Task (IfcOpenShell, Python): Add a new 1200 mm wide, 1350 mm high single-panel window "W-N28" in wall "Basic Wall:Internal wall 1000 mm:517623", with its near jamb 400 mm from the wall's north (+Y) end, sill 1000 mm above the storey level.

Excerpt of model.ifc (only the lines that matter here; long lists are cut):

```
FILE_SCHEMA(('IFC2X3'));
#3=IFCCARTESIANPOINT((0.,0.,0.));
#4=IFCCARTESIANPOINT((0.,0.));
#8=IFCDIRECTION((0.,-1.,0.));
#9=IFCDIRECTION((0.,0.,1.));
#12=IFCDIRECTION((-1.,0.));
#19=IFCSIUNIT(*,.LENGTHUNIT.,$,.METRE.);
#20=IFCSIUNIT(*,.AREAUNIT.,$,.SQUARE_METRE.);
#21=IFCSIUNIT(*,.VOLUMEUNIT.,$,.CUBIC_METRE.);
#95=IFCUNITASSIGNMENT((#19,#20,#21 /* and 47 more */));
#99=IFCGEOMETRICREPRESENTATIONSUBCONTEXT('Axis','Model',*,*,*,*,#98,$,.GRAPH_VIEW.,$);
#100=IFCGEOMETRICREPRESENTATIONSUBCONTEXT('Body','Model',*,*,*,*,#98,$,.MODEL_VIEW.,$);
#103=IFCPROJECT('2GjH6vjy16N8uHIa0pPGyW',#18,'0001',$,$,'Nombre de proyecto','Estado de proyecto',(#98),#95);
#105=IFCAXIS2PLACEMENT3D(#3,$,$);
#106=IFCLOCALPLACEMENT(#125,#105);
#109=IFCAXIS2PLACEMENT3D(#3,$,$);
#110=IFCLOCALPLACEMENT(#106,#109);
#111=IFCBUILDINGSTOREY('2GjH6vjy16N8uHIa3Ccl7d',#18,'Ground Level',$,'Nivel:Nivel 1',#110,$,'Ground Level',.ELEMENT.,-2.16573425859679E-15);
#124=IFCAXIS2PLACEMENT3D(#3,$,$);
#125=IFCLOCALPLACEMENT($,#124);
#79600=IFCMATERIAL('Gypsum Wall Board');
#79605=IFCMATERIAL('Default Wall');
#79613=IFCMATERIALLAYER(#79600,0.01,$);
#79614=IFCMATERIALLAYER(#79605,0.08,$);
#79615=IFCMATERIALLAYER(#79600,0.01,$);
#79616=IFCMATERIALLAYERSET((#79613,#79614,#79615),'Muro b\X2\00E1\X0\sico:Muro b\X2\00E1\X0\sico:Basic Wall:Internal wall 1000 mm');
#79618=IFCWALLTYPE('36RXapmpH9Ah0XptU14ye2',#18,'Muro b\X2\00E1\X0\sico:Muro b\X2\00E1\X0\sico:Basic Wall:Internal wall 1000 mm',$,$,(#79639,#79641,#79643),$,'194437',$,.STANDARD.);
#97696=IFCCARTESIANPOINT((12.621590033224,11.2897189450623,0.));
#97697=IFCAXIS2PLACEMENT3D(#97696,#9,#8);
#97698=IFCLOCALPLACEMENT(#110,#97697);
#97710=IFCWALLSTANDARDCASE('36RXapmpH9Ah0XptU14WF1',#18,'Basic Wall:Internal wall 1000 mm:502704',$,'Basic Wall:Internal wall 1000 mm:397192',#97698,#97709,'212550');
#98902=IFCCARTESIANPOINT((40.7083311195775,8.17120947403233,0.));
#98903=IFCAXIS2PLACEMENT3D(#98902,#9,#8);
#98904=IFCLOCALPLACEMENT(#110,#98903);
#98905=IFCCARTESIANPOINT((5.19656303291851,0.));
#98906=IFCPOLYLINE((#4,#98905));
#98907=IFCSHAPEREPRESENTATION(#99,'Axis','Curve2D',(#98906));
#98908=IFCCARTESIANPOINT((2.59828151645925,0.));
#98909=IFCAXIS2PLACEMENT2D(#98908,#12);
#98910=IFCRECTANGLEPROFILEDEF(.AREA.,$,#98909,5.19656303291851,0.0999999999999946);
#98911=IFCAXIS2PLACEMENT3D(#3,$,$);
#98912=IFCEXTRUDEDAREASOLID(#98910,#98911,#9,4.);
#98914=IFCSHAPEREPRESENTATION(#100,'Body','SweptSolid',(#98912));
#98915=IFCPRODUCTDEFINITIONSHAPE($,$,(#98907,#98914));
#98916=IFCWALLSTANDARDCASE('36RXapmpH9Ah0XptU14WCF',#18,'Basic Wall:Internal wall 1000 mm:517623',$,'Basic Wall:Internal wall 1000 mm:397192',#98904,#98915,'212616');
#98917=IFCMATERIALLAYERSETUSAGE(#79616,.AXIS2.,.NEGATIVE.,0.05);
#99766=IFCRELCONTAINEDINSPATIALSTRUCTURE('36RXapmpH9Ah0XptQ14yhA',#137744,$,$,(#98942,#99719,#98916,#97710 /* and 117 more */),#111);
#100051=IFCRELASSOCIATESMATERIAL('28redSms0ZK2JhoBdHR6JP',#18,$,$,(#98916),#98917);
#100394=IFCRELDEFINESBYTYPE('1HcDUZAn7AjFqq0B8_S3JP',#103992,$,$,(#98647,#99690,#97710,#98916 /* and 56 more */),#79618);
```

```python
import numpy as np
import ifcopenshell
import ifcopenshell.api.feature
import ifcopenshell.api.geometry
import ifcopenshell.api.root
import ifcopenshell.api.spatial
import ifcopenshell.api.type
import ifcopenshell.geom
import ifcopenshell.util.element
import ifcopenshell.util.placement
import ifcopenshell.util.representation
import ifcopenshell.util.shape
import ifcopenshell.util.unit

model = ifcopenshell.open("model.ifc")
unit_scale = ifcopenshell.util.unit.calculate_unit_scale(model)
settings = ifcopenshell.geom.settings()


def volume(element):
    """Net volume in cubic metres, openings subtracted."""
    shape = ifcopenshell.geom.create_shape(settings, element)
    return ifcopenshell.util.shape.get_volume(shape.geometry)


wall = model.by_guid("36RXapmpH9Ah0XptU14WCF")
storey = ifcopenshell.util.element.get_container(wall, ifc_class="IfcBuildingStorey")
context = ifcopenshell.util.representation.get_context(model, "Model", "Body", "MODEL_VIEW")
before = volume(wall)

width, height, from_end, sill = 1.2, 1.35, 0.4, 1  # metres

# The wall runs along its own X axis, and the end named is its -X end.
wall_shape = ifcopenshell.geom.create_shape(settings, wall)
x, y, z = ifcopenshell.util.shape.get_vertices(wall_shape.geometry).T
start = x.min() + from_end
face, thickness = float(y.min()), float(y.max() - y.min())
wall_matrix = ifcopenshell.util.placement.get_local_placement(wall.ObjectPlacement)
level = ifcopenshell.util.placement.get_local_placement(storey.ObjectPlacement)[2, 3]


def in_wall(x, y):
    """Placement at x, y metres in the wall's axes, at sill height."""
    matrix = wall_matrix.copy()
    matrix[:, 3] = wall_matrix @ np.array([x / unit_scale, y / unit_scale, 0.0, 1.0])
    matrix[2, 3] = level + sill / unit_scale
    return matrix


# Opening: a box that overshoots both wall faces by 50 mm.
opening = ifcopenshell.api.root.create_entity(model, ifc_class="IfcOpeningElement")
box = ifcopenshell.api.geometry.add_wall_representation(
    model, context=context, length=width, height=height, thickness=thickness + 0.1
)
ifcopenshell.api.geometry.assign_representation(model, product=opening, representation=box)
ifcopenshell.api.geometry.edit_object_placement(model, product=opening, matrix=in_wall(start, face - 0.05), is_si=False)
ifcopenshell.api.feature.add_feature(model, feature=opening, element=wall)

window = ifcopenshell.api.root.create_entity(model, ifc_class="IfcWindow", name="W-N28")
window.OverallWidth, window.OverallHeight = width / unit_scale, height / unit_scale
body = ifcopenshell.api.geometry.add_window_representation(
    model,
    context=context,
    overall_width=window.OverallWidth,
    overall_height=window.OverallHeight,
    partition_type="SINGLE_PANEL",
)
ifcopenshell.api.geometry.assign_representation(model, product=window, representation=body)
ifcopenshell.api.spatial.assign_container(model, products=[window], relating_structure=storey)
fills = ifcopenshell.api.feature.add_filling(model, opening=opening, element=window)
fills.OwnerHistory = window.OwnerHistory  # required in IFC2X3

# IFC2X3 keeps the operation on the window style.
style = ifcopenshell.api.root.create_entity(model, ifc_class="IfcWindowStyle", name="W-N28")
style.OperationType, style.ConstructionType = "SINGLE_PANEL", "NOTDEFINED"
style.ParameterTakesPrecedence = style.Sizeable = False
ifcopenshell.api.type.assign_type(model, related_objects=[window], relating_type=style)

# Centre the window in the wall's thickness.
ifcopenshell.api.geometry.edit_object_placement(model, product=window, matrix=in_wall(start, face), is_si=False)
window_shape = ifcopenshell.geom.create_shape(settings, window)
depth = ifcopenshell.util.shape.get_vertices(window_shape.geometry)[:, 1]
offset = face + thickness / 2 - (depth.min() + depth.max()) / 2
ifcopenshell.api.geometry.edit_object_placement(model, product=window, matrix=in_wall(start, offset), is_si=False)

after = volume(wall)

print(f"wall volume {before:.3f} -> {after:.3f} m3")

model.write("model_v2.ifc")
```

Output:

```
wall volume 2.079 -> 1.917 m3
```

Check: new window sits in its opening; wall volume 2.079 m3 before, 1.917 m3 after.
